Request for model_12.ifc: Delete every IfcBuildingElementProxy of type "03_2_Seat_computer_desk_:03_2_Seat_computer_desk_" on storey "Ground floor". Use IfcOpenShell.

First a look at what the model holds.

```python
import ifcopenshell
import ifcopenshell.util.element

model = ifcopenshell.open("model_12.ifc")
print(model.schema)
storey = next(s for s in model.by_type("IfcBuildingStorey") if s.Name == "Ground floor")
proxies = [e for e in ifcopenshell.util.element.get_decomposition(storey) if e.is_a("IfcBuildingElementProxy")]
seen = {}
for e in proxies:
    element_type = ifcopenshell.util.element.get_type(e)
    name = element_type.Name if element_type not in (None, e) else None
    seen[name] = seen.get(name, 0) + 1
for name, count in sorted(seen.items(), key=str):
    print(count, "x", name)
```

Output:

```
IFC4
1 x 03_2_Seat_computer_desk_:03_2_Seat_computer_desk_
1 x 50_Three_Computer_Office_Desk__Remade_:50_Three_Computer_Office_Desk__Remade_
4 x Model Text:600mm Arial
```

```python
import ifcopenshell
import ifcopenshell.api.root
import ifcopenshell.util.element

model = ifcopenshell.open("model_12.ifc")

storey = next(s for s in model.by_type("IfcBuildingStorey") if s.Name == "Ground floor")
proxies = [e for e in ifcopenshell.util.element.get_decomposition(storey) if e.is_a("IfcBuildingElementProxy")]
targets = [e for e in proxies if (t := ifcopenshell.util.element.get_type(e)) not in (None, e) and t.Name == "03_2_Seat_computer_desk_:03_2_Seat_computer_desk_"]

for e in targets:
    ifcopenshell.api.root.remove_product(model, product=e)
print(len(targets), "removed")

model.write("model_12_rev.ifc")
```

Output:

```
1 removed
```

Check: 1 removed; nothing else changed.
